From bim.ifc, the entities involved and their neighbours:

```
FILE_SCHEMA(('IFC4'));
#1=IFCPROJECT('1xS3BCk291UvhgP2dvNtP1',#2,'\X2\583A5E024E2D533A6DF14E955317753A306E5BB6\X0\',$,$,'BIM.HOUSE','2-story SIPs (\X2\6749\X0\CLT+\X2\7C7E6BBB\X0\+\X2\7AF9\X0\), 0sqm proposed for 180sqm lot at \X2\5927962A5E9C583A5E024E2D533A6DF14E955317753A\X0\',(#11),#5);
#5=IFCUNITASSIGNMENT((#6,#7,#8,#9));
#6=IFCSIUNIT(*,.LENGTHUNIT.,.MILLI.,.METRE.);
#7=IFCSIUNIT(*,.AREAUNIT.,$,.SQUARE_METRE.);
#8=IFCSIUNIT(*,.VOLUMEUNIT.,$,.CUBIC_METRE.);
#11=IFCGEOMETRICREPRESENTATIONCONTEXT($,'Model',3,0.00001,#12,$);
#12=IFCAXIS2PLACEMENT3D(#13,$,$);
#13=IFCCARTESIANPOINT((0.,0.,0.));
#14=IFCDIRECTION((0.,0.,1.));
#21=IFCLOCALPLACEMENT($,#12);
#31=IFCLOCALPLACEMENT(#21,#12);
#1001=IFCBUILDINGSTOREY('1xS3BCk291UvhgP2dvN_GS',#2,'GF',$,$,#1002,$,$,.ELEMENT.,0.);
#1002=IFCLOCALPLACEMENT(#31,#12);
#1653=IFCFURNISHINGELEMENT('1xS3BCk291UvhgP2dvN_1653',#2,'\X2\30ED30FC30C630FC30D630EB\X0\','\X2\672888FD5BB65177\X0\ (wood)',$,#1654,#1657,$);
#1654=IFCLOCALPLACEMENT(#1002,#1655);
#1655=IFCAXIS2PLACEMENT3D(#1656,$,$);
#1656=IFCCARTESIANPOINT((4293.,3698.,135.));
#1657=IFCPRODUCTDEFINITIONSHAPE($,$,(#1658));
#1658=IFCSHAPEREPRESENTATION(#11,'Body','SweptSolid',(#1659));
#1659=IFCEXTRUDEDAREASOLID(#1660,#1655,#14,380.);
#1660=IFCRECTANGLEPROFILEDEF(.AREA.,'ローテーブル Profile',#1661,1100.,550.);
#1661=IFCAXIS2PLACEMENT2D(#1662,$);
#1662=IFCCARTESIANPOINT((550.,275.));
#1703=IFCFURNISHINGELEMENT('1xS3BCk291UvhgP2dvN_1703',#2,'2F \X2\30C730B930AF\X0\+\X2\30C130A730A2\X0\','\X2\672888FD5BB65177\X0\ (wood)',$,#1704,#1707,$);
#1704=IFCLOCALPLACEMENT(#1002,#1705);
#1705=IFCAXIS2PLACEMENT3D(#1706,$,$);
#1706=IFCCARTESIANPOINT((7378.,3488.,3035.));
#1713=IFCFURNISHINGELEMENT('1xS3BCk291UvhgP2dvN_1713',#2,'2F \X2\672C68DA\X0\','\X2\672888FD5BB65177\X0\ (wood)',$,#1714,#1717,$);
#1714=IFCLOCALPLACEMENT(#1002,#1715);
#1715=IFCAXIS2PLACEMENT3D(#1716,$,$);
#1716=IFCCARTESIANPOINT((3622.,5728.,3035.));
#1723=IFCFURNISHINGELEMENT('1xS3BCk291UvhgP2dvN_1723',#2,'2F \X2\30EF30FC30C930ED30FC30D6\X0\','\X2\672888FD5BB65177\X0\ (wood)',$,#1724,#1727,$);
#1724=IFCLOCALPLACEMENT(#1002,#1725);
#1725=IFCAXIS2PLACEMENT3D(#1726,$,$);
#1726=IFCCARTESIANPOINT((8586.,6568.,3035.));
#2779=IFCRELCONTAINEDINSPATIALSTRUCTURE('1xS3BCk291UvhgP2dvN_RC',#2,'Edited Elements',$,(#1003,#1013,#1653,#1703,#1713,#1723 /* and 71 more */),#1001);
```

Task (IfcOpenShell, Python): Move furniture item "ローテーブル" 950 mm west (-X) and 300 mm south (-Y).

```python
import ifcopenshell
import ifcopenshell.api.geometry
import ifcopenshell.util.placement

model = ifcopenshell.open("bim.ifc")

item = model.by_guid("1xS3BCk291UvhgP2dvN_1653")
matrix = ifcopenshell.util.placement.get_local_placement(item.ObjectPlacement)
matrix[0, 3] -= 950.0
matrix[1, 3] -= 300.0
ifcopenshell.api.geometry.edit_object_placement(model, product=item, matrix=matrix, is_si=False)

print(ifcopenshell.util.placement.get_local_placement(item.ObjectPlacement).round(3) + 0.0)

model.write("bim_v2.ifc")
```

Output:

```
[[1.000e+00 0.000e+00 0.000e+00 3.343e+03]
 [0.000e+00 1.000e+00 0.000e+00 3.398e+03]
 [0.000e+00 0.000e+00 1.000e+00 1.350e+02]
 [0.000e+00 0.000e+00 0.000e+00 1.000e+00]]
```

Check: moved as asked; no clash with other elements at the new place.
